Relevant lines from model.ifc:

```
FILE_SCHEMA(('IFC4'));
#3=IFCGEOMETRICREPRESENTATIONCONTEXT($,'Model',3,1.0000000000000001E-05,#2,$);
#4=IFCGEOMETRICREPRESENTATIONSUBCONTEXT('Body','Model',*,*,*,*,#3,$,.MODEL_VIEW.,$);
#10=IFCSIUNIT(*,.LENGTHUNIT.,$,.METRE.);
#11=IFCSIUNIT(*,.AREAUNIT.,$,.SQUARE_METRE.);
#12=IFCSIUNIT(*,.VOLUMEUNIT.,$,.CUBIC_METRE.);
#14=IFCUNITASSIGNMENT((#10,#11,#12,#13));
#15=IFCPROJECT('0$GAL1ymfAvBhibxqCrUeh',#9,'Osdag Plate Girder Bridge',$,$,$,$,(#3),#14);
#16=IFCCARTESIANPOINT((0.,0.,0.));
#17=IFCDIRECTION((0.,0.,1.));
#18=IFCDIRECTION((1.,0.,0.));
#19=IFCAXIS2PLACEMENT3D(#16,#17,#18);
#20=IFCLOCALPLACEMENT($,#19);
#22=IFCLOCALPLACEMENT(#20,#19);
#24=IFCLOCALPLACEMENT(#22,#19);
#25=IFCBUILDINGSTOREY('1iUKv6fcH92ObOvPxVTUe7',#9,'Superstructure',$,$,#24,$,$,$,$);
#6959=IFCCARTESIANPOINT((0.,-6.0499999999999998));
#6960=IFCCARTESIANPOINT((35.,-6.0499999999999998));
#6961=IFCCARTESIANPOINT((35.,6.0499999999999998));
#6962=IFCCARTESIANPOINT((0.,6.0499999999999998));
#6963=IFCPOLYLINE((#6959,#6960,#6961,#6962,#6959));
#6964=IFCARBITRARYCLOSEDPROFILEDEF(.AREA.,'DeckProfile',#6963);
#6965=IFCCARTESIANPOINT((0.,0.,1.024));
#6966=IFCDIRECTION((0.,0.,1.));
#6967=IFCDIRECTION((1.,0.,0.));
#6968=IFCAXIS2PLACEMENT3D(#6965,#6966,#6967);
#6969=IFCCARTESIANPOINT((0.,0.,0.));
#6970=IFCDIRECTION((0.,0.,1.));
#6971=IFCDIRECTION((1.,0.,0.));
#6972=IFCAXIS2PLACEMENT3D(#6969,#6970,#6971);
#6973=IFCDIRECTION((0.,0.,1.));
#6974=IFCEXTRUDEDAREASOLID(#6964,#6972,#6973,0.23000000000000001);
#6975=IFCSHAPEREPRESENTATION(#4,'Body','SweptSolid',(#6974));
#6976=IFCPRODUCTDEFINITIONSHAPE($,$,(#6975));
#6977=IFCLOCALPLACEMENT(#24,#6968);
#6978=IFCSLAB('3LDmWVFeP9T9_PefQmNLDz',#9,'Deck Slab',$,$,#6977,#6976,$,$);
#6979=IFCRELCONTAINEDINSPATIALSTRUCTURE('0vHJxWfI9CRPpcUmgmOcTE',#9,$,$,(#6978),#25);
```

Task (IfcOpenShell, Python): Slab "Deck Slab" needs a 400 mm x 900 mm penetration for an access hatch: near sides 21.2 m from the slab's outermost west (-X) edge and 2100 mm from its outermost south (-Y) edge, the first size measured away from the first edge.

```python
import numpy as np
import ifcopenshell
import ifcopenshell.api.feature
import ifcopenshell.api.geometry
import ifcopenshell.api.root
import ifcopenshell.geom
import ifcopenshell.util.placement
import ifcopenshell.util.representation
import ifcopenshell.util.shape
import ifcopenshell.util.unit

model = ifcopenshell.open("model.ifc")
unit_scale = ifcopenshell.util.unit.calculate_unit_scale(model)
settings = ifcopenshell.geom.settings()


def volume(element):
    """Net volume in cubic metres, openings subtracted."""
    shape = ifcopenshell.geom.create_shape(settings, element)
    return ifcopenshell.util.shape.get_volume(shape.geometry)


slab = model.by_id(6978)
before = volume(slab)

# Extent in the slab's own axes, in metres. The edges named are its -X and -Y sides.
slab_shape = ifcopenshell.geom.create_shape(settings, slab)
vertices = ifcopenshell.util.shape.get_vertices(slab_shape.geometry)
x_min, y_min, bottom = vertices.min(axis=0)
top = vertices[:, 2].max()

opening = ifcopenshell.api.root.create_entity(model, ifc_class="IfcOpeningElement", name="Access hatch opening", predefined_type="OPENING")
context = ifcopenshell.util.representation.get_context(model, "Model", "Body", "MODEL_VIEW")
width, depth = 0.4, 0.9
outline = [(0.0, 0.0), (width, 0.0), (width, depth), (0.0, depth), (0.0, 0.0)]
# Overshoot both faces by 50 mm so the cut is clean.
shape = ifcopenshell.api.geometry.add_slab_representation(
    model, context=context, depth=top - bottom + 0.1, polyline=outline
)
ifcopenshell.api.geometry.assign_representation(model, product=opening, representation=shape)

matrix = ifcopenshell.util.placement.get_local_placement(slab.ObjectPlacement)
matrix[:, 3] = matrix @ np.append(np.array([x_min + 21.2, y_min + 2.1, bottom - 0.05]) / unit_scale, 1.0)
ifcopenshell.api.geometry.edit_object_placement(model, product=opening, matrix=matrix, is_si=False)
ifcopenshell.api.feature.add_feature(model, feature=opening, element=slab)

after = volume(slab)

print(f"slab volume {before:.3f} -> {after:.3f} m3")

model.write("model_edited.ifc")
```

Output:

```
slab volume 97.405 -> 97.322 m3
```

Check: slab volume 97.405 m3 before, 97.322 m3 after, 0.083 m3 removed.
